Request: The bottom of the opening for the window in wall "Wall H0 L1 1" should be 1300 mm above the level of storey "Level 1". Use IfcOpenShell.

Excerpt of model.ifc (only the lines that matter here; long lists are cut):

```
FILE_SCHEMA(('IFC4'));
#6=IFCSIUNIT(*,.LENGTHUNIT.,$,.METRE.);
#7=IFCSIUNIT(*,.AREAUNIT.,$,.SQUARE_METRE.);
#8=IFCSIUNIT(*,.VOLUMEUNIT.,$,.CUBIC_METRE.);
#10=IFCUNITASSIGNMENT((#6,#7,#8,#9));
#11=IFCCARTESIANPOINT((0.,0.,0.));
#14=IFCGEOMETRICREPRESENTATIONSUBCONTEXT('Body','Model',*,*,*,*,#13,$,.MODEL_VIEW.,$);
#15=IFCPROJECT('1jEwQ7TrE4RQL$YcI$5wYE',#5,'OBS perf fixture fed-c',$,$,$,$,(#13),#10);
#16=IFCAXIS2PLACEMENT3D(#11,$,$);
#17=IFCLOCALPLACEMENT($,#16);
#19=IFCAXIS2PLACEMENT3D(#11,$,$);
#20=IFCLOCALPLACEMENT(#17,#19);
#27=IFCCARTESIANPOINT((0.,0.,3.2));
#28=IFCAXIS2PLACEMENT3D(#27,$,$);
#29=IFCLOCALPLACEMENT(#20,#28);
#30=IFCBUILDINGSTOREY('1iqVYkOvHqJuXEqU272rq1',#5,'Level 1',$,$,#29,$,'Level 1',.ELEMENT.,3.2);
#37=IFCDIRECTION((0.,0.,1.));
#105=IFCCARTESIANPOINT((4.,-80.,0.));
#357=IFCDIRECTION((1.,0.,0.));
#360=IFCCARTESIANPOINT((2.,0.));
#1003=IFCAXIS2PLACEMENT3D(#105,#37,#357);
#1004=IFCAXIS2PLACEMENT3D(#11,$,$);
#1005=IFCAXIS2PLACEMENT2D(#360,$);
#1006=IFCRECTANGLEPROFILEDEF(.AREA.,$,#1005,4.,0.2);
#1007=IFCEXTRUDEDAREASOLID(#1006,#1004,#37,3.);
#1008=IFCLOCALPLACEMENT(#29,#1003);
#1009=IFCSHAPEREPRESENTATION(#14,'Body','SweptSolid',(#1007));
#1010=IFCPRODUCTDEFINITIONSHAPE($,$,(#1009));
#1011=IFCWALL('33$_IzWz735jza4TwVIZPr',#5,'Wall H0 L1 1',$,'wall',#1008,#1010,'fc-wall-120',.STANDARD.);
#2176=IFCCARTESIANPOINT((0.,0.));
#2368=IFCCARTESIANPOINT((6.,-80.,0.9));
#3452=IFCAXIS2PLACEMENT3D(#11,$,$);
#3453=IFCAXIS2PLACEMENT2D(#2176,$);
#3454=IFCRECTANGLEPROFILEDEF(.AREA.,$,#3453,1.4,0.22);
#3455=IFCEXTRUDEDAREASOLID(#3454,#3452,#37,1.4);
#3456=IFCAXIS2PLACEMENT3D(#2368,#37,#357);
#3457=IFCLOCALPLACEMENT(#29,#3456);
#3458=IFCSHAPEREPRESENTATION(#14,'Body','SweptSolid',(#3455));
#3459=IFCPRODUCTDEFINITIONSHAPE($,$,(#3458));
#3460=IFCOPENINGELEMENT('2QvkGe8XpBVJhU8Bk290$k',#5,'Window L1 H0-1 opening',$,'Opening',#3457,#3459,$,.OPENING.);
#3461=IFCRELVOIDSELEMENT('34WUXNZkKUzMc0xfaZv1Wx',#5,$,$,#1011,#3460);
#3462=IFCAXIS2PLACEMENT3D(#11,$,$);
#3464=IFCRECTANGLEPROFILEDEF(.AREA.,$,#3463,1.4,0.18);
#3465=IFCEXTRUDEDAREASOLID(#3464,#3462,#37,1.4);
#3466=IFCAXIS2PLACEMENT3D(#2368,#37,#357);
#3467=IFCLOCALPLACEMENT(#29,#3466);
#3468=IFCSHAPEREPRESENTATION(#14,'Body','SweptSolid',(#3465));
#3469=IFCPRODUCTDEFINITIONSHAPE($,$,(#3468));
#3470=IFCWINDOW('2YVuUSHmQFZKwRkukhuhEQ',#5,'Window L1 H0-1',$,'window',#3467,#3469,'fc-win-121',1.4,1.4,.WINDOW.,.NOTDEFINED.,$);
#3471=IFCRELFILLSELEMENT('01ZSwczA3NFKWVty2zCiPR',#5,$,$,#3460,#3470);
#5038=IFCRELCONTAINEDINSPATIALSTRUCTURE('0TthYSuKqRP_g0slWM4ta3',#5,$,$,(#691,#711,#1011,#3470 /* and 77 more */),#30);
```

```python
import numpy as np
import ifcopenshell
import ifcopenshell.api.geometry
import ifcopenshell.geom
import ifcopenshell.util.element
import ifcopenshell.util.placement
import ifcopenshell.util.shape
import ifcopenshell.util.unit

model = ifcopenshell.open("model.ifc")
unit_scale = ifcopenshell.util.unit.calculate_unit_scale(model)

window = model.by_guid("2YVuUSHmQFZKwRkukhuhEQ")
opening = window.FillsVoids[0].RelatingOpeningElement
storey = ifcopenshell.util.element.get_container(window, ifc_class="IfcBuildingStorey")
level = ifcopenshell.util.placement.get_local_placement(storey.ObjectPlacement)[2, 3]

# The opening's origin need not be at the sill, so measure its lowest point.
shape = ifcopenshell.geom.create_shape(ifcopenshell.geom.settings(), opening)
bottom = ifcopenshell.util.shape.get_shape_bottom_elevation(shape, shape.geometry) / unit_scale
dz = level + 1.3 / unit_scale - bottom

shift = np.array([0.0, 0.0, dz])
# The window is not placed relative to its opening, so move both.
for product in (opening, window):
    matrix = ifcopenshell.util.placement.get_local_placement(product.ObjectPlacement)
    matrix[:3, 3] += shift
    ifcopenshell.api.geometry.edit_object_placement(model, product=product, matrix=matrix, is_si=False)

print(f"moved by {dz * unit_scale:+.3f} m")

model.write("model_updated.ifc")
```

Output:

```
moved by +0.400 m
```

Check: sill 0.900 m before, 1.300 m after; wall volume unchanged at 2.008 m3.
